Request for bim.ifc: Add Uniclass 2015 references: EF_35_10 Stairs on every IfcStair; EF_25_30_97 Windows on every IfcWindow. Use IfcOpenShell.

First a look at what the model holds.

```python
import ifcopenshell

model = ifcopenshell.open("bim.ifc")
print(model.schema)
print("classifications:", [c.Name for c in model.by_type("IfcClassification")])
for ifc_class in ("IfcDoor", "IfcRoof", "IfcStair", "IfcWall", "IfcWindow"):
    print(ifc_class, len(model.by_type(ifc_class)))
```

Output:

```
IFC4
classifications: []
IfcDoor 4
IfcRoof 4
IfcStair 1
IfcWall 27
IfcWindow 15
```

```python
import ifcopenshell
import ifcopenshell.api.classification

model = ifcopenshell.open("bim.ifc")

system = ifcopenshell.api.classification.add_classification(model, classification="Uniclass 2015")

codes = {
    "IfcStair": ("EF_35_10", "Stairs"),
    "IfcWindow": ("EF_25_30_97", "Windows"),
}
for ifc_class, (code, name) in codes.items():
    products = model.by_type(ifc_class)
    ifcopenshell.api.classification.add_reference(
        model, products=products, classification=system, identification=code, name=name
    )
    print(code, len(products))

model.write("bim_v2.ifc")
```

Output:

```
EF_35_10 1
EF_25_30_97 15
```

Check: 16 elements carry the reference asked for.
